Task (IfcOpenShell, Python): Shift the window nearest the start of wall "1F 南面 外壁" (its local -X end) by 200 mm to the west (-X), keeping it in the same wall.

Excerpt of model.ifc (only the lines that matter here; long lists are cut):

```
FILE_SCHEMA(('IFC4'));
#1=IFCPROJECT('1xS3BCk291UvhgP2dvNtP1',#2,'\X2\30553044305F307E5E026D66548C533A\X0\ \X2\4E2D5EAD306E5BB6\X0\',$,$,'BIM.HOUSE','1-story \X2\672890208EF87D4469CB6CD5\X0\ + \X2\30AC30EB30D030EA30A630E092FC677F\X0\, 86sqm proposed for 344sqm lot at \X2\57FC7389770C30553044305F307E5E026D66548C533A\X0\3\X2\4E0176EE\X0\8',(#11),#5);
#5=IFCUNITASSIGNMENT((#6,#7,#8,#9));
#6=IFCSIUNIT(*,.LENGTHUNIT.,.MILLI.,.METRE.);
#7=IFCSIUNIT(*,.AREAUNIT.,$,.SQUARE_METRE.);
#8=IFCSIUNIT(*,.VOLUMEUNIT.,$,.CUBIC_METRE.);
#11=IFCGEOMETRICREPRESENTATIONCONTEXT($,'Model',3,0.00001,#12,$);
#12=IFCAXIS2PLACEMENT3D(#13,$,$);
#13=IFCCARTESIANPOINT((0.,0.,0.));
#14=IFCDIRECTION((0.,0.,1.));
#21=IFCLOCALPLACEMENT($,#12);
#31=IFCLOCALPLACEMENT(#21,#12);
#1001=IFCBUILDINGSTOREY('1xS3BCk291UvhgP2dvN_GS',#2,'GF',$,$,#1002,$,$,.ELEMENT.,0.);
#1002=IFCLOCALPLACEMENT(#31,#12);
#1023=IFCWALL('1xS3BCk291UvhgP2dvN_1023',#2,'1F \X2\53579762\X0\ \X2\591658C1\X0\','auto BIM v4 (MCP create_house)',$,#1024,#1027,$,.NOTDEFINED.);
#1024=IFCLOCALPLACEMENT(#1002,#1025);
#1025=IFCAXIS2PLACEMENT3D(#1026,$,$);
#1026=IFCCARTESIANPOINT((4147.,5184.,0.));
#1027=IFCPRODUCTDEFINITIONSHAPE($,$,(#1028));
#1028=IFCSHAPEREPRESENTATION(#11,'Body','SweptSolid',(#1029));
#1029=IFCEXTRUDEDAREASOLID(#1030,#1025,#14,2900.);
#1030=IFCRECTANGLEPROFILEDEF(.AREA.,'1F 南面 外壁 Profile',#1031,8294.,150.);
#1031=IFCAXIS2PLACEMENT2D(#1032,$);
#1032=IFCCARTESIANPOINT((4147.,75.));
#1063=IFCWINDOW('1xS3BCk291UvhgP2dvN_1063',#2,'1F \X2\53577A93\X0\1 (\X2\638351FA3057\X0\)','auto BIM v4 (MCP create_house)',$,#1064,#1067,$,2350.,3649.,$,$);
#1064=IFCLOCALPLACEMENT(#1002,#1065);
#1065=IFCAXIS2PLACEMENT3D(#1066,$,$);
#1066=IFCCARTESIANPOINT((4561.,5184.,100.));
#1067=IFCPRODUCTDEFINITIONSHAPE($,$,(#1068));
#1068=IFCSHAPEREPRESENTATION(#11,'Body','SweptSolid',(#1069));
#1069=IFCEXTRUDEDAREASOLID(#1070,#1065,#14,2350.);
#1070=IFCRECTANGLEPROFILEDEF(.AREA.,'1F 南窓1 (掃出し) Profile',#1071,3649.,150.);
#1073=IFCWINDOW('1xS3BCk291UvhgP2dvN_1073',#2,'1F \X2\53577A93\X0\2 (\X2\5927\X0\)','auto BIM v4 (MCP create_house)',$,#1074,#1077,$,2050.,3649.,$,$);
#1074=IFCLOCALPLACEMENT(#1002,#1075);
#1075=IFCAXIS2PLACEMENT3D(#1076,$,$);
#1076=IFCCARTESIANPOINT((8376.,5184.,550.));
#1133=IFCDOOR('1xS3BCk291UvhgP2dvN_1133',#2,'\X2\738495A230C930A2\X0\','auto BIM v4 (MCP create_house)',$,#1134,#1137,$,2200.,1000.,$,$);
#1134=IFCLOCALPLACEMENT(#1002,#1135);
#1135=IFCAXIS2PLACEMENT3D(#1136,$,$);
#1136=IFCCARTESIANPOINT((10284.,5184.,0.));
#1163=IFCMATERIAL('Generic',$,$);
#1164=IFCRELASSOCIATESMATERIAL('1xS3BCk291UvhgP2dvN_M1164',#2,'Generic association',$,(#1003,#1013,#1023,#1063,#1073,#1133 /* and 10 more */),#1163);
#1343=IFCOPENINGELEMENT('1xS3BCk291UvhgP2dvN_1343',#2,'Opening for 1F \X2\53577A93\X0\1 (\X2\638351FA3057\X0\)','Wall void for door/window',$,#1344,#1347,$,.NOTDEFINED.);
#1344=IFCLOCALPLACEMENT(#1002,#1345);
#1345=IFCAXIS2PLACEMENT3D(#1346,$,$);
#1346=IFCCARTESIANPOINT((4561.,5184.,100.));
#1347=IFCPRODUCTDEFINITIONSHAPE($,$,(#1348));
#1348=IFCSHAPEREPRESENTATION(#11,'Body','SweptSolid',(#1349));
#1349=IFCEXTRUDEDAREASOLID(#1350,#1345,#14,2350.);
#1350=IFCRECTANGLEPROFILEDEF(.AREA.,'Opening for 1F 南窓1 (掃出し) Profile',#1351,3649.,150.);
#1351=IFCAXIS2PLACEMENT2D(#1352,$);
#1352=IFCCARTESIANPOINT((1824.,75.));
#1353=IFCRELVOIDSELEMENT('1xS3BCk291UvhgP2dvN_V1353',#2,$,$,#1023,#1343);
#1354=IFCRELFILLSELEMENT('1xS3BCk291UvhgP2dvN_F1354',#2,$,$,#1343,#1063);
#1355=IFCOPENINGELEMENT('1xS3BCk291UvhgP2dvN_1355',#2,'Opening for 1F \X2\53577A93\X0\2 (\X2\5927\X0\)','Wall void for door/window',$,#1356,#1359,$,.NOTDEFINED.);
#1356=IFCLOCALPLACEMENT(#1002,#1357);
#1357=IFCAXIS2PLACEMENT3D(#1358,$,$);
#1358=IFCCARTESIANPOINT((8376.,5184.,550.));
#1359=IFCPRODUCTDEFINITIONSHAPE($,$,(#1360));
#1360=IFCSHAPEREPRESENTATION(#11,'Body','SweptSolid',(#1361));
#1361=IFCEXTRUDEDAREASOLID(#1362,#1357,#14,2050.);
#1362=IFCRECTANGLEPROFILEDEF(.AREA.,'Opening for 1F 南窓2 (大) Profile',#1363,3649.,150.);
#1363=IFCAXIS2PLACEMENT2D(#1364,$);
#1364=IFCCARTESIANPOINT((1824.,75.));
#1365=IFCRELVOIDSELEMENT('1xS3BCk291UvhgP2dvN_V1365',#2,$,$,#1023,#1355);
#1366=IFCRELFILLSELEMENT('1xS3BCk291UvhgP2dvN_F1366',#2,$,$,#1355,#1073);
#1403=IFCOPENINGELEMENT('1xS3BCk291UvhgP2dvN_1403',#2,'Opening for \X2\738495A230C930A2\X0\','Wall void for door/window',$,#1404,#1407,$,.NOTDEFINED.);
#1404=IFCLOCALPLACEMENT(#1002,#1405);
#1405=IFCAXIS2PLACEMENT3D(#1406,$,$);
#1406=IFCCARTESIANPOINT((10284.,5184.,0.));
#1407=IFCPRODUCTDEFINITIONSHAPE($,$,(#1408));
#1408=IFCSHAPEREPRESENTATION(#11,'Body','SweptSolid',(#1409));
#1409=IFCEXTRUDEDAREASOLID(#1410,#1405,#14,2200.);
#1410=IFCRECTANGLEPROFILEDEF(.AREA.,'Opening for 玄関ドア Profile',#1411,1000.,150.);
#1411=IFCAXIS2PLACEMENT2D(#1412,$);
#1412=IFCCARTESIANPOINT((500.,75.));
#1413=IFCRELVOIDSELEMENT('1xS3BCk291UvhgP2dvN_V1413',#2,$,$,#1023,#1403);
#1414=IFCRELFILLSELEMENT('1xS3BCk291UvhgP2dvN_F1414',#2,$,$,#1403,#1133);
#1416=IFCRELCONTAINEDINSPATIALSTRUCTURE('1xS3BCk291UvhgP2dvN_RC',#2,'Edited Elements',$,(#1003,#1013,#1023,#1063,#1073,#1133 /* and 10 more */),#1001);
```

```python
import ifcopenshell
import ifcopenshell.api.geometry
import ifcopenshell.util.placement

model = ifcopenshell.open("model.ifc")

window = model.by_id(1063)
opening = window.FillsVoids[0].RelatingOpeningElement
wall = opening.VoidsElements[0].RelatingBuildingElement

wall_matrix = ifcopenshell.util.placement.get_local_placement(wall.ObjectPlacement)
shift = wall_matrix[:3, 0] * -200.0
before = ifcopenshell.util.placement.get_local_placement(window.ObjectPlacement)[:3, 3].copy()

# The window is not placed relative to its opening, so move both.
for product in (opening, window):
    matrix = ifcopenshell.util.placement.get_local_placement(product.ObjectPlacement)
    matrix[:3, 3] += shift
    ifcopenshell.api.geometry.edit_object_placement(model, product=product, matrix=matrix, is_si=False)

after = ifcopenshell.util.placement.get_local_placement(window.ObjectPlacement)[:3, 3]
print("window moved by", (after - before).round(3) + 0.0)

model.write("model-out.ifc")
```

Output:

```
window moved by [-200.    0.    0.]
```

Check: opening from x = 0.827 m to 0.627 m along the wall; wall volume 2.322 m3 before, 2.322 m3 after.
